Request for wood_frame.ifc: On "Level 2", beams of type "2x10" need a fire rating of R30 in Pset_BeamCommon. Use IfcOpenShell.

First a look at what the model holds.

```python
import ifcopenshell
import ifcopenshell.util.element

model = ifcopenshell.open("wood_frame.ifc")
print(model.schema)
storey = next(s for s in model.by_type("IfcBuildingStorey") if s.Name == "Level 2")
beams = [e for e in ifcopenshell.util.element.get_decomposition(storey) if e.is_a("IfcBeam")]
seen = {}
for e in beams:
    element_type = ifcopenshell.util.element.get_type(e)
    key = (element_type.Name if element_type != e and element_type else None, ifcopenshell.util.element.get_pset(e, "Pset_BeamCommon", "FireRating"))
    seen[key] = seen.get(key, 0) + 1
for (name, value), count in sorted(seen.items(), key=str):
    print(count, "x", name, "|", value)
```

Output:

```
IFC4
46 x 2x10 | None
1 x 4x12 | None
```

```python
import ifcopenshell
import ifcopenshell.api.pset
import ifcopenshell.util.element

model = ifcopenshell.open("wood_frame.ifc")

storey = next(s for s in model.by_type("IfcBuildingStorey") if s.Name == "Level 2")
beams = [e for e in ifcopenshell.util.element.get_decomposition(storey) if e.is_a("IfcBeam")]

count = 0
for e in beams:
    element_type = ifcopenshell.util.element.get_type(e)
    if element_type in (None, e) or element_type.Name != "2x10":
        continue
    # add_pset returns the element's existing set when there is one.
    pset = ifcopenshell.api.pset.add_pset(model, product=e, name="Pset_BeamCommon")
    ifcopenshell.api.pset.edit_pset(model, pset=pset, properties={"FireRating": "R30"})
    count += 1

print(count, "beams updated")

model.write("wood_frame_rev.ifc")
```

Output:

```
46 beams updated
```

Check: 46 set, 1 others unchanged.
